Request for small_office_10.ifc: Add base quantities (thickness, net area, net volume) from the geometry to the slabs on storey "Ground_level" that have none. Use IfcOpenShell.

First a look at what the model holds.

```python
import ifcopenshell
import ifcopenshell.util.element
import ifcopenshell.util.unit

model = ifcopenshell.open("small_office_10.ifc")
print(model.schema)
for unit_type in ("LENGTHUNIT", "AREAUNIT", "VOLUMEUNIT"):
    print(unit_type, ifcopenshell.util.unit.calculate_unit_scale(model, unit_type))
storey = next(s for s in model.by_type("IfcBuildingStorey") if s.Name == "Ground_level")
slabs = [e for e in ifcopenshell.util.element.get_decomposition(storey) if e.is_a("IfcSlab")]
for e in sorted(slabs, key=lambda e: e.id()):
    print(e.id(), e.is_a(), e.Name, list(ifcopenshell.util.element.get_psets(e, qtos_only=True)), sep=" | ")
```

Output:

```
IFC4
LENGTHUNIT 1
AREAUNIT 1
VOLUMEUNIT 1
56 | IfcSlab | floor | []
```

```python
import ifcopenshell
import ifcopenshell.api.pset
import ifcopenshell.geom
import ifcopenshell.util.element
import ifcopenshell.util.shape
import ifcopenshell.util.unit

model = ifcopenshell.open("small_office_10.ifc")
unit_scale = ifcopenshell.util.unit.calculate_unit_scale(model)
area_scale = ifcopenshell.util.unit.calculate_unit_scale(model, "AREAUNIT")
volume_scale = ifcopenshell.util.unit.calculate_unit_scale(model, "VOLUMEUNIT")
settings = ifcopenshell.geom.settings()

storey = next(s for s in model.by_type("IfcBuildingStorey") if s.Name == "Ground_level")
slabs = [e for e in ifcopenshell.util.element.get_decomposition(storey) if e.is_a("IfcSlab")]

for e in sorted(slabs, key=lambda e: e.id()):
    if ifcopenshell.util.element.get_psets(e, qtos_only=True, should_inherit=False):
        continue
    # Geometry comes back in metres, in the element's own axes.
    shape = ifcopenshell.geom.create_shape(settings, e)
    values = {
        "Width": ifcopenshell.util.shape.get_z(shape.geometry) / unit_scale,
        "NetArea": ifcopenshell.util.shape.get_footprint_area(shape.geometry) / area_scale,
        "NetVolume": ifcopenshell.util.shape.get_volume(shape.geometry) / volume_scale,
    }
    qto = ifcopenshell.api.pset.add_qto(model, product=e, name="Qto_SlabBaseQuantities")
    ifcopenshell.api.pset.edit_qto(model, qto=qto, properties=values)
    print(e.id(), {k: round(v, 3) for k, v in values.items()})

model.write("small_office_10_edited.ifc")
```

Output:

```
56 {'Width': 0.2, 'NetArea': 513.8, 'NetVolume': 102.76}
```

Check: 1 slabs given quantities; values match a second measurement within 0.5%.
